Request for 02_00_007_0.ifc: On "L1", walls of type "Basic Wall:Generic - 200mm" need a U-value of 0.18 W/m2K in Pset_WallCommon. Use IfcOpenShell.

First a look at what the model holds.

```python
import ifcopenshell
import ifcopenshell.util.element

model = ifcopenshell.open("02_00_007_0.ifc")
print(model.schema)
storey = next(s for s in model.by_type("IfcBuildingStorey") if s.Name == "L1")
walls = [e for e in ifcopenshell.util.element.get_decomposition(storey) if e.is_a("IfcWall")]
seen = {}
for e in walls:
    element_type = ifcopenshell.util.element.get_type(e)
    key = (element_type.Name if element_type != e and element_type else None, ifcopenshell.util.element.get_pset(e, "Pset_WallCommon", "ThermalTransmittance"))
    seen[key] = seen.get(key, 0) + 1
for (name, value), count in sorted(seen.items(), key=str):
    print(count, "x", name, "|", value)
```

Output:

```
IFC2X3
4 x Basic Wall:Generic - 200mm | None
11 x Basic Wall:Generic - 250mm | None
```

```python
import ifcopenshell
import ifcopenshell.api.pset
import ifcopenshell.util.element

model = ifcopenshell.open("02_00_007_0.ifc")

storey = next(s for s in model.by_type("IfcBuildingStorey") if s.Name == "L1")
walls = [e for e in ifcopenshell.util.element.get_decomposition(storey) if e.is_a("IfcWall")]

count = 0
for e in walls:
    element_type = ifcopenshell.util.element.get_type(e)
    if element_type in (None, e) or element_type.Name != "Basic Wall:Generic - 200mm":
        continue
    # add_pset returns the element's existing set when there is one.
    pset = ifcopenshell.api.pset.add_pset(model, product=e, name="Pset_WallCommon")
    ifcopenshell.api.pset.edit_pset(model, pset=pset, properties={"ThermalTransmittance": 0.18})
    count += 1

print(count, "walls updated")

model.write("02_00_007_0_edited.ifc")
```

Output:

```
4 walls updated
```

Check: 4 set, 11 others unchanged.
